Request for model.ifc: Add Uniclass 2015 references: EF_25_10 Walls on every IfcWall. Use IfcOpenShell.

First a look at what the model holds.

```python
import ifcopenshell

model = ifcopenshell.open("model.ifc")
print(model.schema)
print("classifications:", [c.Name for c in model.by_type("IfcClassification")])
for ifc_class in ("IfcDoor", "IfcRoof", "IfcStair", "IfcWall", "IfcWindow"):
    print(ifc_class, len(model.by_type(ifc_class)))
```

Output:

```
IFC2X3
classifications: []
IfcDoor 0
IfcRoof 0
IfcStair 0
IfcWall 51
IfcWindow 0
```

```python
import ifcopenshell
import ifcopenshell.api.classification

model = ifcopenshell.open("model.ifc")

# IFC2X3 requires Source and Edition and has no link from the project to the system.
system = model.create_entity("IfcClassification", Source="NBS", Edition="2015", Name="Uniclass 2015")

codes = {
    "IfcWall": ("EF_25_10", "Walls"),
}
for ifc_class, (code, name) in codes.items():
    products = model.by_type(ifc_class)
    ifcopenshell.api.classification.add_reference(
        model, products=products, classification=system, identification=code, name=name
    )
    print(code, len(products))

model.write("model_edited.ifc")
```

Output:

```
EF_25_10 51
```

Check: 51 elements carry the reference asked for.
